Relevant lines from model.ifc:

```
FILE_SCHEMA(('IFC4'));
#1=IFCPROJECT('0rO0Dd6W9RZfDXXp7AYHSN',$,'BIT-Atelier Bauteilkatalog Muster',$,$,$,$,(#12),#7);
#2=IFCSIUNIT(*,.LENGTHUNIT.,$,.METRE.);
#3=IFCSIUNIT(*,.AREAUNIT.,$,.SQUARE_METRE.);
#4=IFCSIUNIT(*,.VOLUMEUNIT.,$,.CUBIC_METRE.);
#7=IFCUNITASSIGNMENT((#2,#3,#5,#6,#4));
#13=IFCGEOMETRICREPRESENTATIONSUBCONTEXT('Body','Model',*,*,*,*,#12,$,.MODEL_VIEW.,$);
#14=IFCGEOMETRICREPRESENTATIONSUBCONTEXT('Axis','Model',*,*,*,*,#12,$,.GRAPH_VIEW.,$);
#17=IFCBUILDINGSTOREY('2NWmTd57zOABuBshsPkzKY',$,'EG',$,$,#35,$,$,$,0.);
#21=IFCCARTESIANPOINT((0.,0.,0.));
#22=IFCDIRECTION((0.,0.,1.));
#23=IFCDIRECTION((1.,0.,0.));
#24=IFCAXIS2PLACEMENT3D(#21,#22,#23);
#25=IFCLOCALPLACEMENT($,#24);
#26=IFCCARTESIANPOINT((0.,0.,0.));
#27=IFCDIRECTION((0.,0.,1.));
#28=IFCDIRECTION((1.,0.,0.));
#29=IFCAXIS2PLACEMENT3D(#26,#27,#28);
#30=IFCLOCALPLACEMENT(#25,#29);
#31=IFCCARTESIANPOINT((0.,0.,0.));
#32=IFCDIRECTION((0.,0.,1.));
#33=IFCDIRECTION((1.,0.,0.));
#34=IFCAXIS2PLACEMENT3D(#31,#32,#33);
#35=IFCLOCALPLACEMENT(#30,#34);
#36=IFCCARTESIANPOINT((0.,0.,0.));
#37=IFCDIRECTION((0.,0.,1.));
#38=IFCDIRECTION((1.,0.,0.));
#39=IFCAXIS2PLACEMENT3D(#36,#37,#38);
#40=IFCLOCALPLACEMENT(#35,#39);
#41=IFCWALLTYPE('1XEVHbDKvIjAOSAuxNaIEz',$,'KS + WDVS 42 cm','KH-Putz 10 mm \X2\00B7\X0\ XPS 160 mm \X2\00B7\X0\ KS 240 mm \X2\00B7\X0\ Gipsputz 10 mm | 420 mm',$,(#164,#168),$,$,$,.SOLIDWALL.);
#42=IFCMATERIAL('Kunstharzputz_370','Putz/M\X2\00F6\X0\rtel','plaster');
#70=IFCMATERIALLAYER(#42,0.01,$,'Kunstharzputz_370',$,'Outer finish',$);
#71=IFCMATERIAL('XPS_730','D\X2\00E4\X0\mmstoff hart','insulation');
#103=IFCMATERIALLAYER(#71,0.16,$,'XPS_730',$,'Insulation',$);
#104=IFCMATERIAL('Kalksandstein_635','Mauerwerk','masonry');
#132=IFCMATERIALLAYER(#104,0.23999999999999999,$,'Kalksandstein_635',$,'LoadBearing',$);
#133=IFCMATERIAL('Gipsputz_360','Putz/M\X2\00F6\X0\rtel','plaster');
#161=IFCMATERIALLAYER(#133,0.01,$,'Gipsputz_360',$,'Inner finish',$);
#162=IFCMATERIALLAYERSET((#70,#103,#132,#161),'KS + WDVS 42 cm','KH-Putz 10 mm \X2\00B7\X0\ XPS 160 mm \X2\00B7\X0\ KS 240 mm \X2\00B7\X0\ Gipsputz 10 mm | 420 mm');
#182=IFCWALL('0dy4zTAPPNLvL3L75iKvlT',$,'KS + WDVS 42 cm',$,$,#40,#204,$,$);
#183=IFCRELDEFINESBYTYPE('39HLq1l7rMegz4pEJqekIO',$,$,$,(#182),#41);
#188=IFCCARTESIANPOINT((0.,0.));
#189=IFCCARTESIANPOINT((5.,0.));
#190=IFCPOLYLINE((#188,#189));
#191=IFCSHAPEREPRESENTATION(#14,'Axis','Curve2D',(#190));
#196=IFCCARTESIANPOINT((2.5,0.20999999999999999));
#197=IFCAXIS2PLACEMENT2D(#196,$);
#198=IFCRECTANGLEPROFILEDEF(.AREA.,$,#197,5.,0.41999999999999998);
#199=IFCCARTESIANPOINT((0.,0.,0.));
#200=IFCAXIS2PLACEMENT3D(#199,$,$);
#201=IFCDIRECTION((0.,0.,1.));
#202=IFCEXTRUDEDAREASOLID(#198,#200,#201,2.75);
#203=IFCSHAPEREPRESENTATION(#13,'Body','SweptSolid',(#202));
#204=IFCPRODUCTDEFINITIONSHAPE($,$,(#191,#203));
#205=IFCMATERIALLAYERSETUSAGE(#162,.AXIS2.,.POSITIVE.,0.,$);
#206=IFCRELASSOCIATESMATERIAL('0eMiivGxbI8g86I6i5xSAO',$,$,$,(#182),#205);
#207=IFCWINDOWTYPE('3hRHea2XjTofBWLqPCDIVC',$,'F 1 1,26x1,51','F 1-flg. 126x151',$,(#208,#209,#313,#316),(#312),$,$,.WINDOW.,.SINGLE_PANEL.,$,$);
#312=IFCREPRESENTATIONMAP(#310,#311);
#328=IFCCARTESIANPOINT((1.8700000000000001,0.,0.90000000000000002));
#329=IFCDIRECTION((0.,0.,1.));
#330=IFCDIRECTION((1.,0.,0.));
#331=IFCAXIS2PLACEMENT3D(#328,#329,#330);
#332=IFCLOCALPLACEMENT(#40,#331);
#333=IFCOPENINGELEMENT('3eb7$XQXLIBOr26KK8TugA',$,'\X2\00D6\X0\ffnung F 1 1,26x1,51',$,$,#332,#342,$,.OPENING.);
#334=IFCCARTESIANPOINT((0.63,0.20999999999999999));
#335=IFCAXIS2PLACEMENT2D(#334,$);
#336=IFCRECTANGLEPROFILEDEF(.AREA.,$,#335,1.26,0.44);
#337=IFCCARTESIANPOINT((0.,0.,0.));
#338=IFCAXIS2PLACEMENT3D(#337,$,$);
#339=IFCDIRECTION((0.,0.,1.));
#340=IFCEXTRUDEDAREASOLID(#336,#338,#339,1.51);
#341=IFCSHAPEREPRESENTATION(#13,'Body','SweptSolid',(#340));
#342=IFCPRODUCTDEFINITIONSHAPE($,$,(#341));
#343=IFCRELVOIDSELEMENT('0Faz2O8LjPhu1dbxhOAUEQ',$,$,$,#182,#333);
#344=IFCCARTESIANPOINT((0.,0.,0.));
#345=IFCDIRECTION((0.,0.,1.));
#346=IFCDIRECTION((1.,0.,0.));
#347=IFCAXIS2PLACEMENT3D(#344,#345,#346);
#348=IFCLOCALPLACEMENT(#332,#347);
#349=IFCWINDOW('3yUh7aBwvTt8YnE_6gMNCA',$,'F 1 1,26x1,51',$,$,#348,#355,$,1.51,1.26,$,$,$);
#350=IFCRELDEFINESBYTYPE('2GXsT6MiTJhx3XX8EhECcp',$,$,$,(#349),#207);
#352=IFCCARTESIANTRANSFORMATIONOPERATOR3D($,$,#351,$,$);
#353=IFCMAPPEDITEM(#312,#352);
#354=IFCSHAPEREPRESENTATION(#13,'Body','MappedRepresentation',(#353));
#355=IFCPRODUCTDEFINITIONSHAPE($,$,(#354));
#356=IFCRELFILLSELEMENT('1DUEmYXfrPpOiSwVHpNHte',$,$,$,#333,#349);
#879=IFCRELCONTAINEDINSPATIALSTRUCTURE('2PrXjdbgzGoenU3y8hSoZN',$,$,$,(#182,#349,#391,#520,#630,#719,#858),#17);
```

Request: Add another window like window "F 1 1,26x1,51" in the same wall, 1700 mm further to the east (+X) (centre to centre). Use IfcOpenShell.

```python
import ifcopenshell
import ifcopenshell.api.feature
import ifcopenshell.api.geometry
import ifcopenshell.api.root
import ifcopenshell.geom
import ifcopenshell.util.element
import ifcopenshell.util.placement
import ifcopenshell.util.shape
import ifcopenshell.util.unit

model = ifcopenshell.open("model.ifc")
unit_scale = ifcopenshell.util.unit.calculate_unit_scale(model)
settings = ifcopenshell.geom.settings()


def volume(element):
    """Net volume in cubic metres, openings subtracted."""
    shape = ifcopenshell.geom.create_shape(settings, element)
    return ifcopenshell.util.shape.get_volume(shape.geometry)


window = model.by_guid("3yUh7aBwvTt8YnE_6gMNCA")
opening = window.FillsVoids[0].RelatingOpeningElement
wall = opening.VoidsElements[0].RelatingBuildingElement
before = volume(wall)
shift = ifcopenshell.util.placement.get_local_placement(wall.ObjectPlacement)[:3, 0] * 1.7 / unit_scale

# copy_class copies the void relationship, type, container and properties, but no geometry.
new_opening = ifcopenshell.api.root.copy_class(model, product=opening)
new_opening.Representation = ifcopenshell.util.element.copy_deep(
    model, opening.Representation, exclude=["IfcGeometricRepresentationContext", "IfcRepresentationMap"]
)
new_window = ifcopenshell.api.root.copy_class(model, product=window)
new_window.Representation = ifcopenshell.util.element.copy_deep(
    model, window.Representation, exclude=["IfcGeometricRepresentationContext", "IfcRepresentationMap"]
)
ifcopenshell.api.feature.add_filling(model, opening=new_opening, element=new_window)

for old, new in ((opening, new_opening), (window, new_window)):
    matrix = ifcopenshell.util.placement.get_local_placement(old.ObjectPlacement)
    matrix[:3, 3] += shift
    ifcopenshell.api.geometry.edit_object_placement(model, product=new, matrix=matrix, is_si=False)

after = volume(wall)

print(f"wall volume {before:.3f} -> {after:.3f} m3")

model.write("model-out.ifc")
```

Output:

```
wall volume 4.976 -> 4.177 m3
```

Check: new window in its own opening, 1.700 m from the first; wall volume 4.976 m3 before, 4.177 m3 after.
